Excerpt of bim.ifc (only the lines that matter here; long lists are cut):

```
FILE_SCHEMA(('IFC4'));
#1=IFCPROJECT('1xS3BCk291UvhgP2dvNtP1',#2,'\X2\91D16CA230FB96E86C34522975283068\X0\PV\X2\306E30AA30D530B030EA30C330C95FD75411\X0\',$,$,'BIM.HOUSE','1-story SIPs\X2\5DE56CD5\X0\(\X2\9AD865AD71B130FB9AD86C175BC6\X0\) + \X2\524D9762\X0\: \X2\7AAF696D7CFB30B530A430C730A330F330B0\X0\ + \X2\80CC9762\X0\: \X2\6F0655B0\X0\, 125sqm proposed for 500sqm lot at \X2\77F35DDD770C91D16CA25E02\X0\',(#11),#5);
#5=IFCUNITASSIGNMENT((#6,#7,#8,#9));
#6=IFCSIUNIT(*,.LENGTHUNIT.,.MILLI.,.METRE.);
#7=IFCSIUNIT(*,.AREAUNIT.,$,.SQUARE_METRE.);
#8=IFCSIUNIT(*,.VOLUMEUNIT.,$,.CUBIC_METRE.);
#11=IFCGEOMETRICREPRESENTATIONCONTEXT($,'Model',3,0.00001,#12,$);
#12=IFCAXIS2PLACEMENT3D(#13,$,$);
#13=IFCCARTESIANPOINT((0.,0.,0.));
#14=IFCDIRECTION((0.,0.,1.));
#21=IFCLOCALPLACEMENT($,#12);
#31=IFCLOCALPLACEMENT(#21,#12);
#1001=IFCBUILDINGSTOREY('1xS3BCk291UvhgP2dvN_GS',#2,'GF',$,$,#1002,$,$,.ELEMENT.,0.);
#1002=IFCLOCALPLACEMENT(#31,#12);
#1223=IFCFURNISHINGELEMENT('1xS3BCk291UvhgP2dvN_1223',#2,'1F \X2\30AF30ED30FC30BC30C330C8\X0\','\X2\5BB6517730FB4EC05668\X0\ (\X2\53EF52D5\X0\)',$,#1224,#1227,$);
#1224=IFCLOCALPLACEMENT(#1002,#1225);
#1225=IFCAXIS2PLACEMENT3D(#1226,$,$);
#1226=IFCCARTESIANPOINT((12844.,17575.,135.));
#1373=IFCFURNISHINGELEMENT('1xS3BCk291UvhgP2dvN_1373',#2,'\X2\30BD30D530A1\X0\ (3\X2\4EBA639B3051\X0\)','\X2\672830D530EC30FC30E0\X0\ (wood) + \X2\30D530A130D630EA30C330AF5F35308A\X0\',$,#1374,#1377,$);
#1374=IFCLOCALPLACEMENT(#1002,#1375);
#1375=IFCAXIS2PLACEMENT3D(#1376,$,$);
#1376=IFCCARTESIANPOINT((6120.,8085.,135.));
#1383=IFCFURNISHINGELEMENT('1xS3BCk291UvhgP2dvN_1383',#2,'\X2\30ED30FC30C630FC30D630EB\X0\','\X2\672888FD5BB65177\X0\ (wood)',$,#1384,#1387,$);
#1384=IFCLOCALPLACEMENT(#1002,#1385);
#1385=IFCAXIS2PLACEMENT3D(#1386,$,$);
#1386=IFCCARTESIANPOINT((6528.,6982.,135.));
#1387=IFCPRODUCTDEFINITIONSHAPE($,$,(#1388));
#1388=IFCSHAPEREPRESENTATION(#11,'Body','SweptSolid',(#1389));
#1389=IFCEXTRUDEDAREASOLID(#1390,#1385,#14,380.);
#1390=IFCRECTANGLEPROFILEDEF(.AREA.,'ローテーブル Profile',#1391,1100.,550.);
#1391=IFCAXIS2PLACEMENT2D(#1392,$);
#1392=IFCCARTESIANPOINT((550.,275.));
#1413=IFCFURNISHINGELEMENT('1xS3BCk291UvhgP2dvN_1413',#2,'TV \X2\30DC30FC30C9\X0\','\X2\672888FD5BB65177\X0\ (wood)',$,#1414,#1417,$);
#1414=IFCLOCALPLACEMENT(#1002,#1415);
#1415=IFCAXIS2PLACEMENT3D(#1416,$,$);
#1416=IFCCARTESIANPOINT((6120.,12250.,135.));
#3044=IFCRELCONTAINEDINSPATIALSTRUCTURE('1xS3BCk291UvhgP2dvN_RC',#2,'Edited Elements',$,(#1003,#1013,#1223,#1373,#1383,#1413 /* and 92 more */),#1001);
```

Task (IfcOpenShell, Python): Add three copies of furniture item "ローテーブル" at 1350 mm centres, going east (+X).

```python
import numpy as np
import ifcopenshell
import ifcopenshell.api.geometry
import ifcopenshell.api.root
import ifcopenshell.util.element
import ifcopenshell.util.placement
import ifcopenshell.util.unit

model = ifcopenshell.open("bim.ifc")
unit_scale = ifcopenshell.util.unit.calculate_unit_scale(model)


def reuse_history(source, copy):
    """copy_class also copies each property set's owner history, people and application; keep the originals."""
    for rel in copy.IsDefinedBy:
        if rel.is_a("IfcRelDefinesByProperties") and (history := rel.RelatingPropertyDefinition.OwnerHistory):
            rel.RelatingPropertyDefinition.OwnerHistory = source.OwnerHistory
            ifcopenshell.util.element.remove_deep2(model, history)


source = model.by_id(1383)
base = ifcopenshell.util.placement.get_local_placement(source.ObjectPlacement)
step = np.array([1.0, 0.0, 0.0]) * 1.35 / unit_scale

for i in range(1, 4):
    copy = ifcopenshell.api.root.copy_class(model, product=source)
    copy.Representation = ifcopenshell.util.element.copy_deep(
        model, source.Representation, exclude=["IfcGeometricRepresentationContext", "IfcRepresentationMap"]
    )
    reuse_history(source, copy)
    matrix = base.copy()
    matrix[:3, 3] += i * step
    print("added at", matrix[:3, 3].round(3) + 0.0)
    ifcopenshell.api.geometry.edit_object_placement(model, product=copy, matrix=matrix, is_si=False)

model.write("bim-out.ifc")
```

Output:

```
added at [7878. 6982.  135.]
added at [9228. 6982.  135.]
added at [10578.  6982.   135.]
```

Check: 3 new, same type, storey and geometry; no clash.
